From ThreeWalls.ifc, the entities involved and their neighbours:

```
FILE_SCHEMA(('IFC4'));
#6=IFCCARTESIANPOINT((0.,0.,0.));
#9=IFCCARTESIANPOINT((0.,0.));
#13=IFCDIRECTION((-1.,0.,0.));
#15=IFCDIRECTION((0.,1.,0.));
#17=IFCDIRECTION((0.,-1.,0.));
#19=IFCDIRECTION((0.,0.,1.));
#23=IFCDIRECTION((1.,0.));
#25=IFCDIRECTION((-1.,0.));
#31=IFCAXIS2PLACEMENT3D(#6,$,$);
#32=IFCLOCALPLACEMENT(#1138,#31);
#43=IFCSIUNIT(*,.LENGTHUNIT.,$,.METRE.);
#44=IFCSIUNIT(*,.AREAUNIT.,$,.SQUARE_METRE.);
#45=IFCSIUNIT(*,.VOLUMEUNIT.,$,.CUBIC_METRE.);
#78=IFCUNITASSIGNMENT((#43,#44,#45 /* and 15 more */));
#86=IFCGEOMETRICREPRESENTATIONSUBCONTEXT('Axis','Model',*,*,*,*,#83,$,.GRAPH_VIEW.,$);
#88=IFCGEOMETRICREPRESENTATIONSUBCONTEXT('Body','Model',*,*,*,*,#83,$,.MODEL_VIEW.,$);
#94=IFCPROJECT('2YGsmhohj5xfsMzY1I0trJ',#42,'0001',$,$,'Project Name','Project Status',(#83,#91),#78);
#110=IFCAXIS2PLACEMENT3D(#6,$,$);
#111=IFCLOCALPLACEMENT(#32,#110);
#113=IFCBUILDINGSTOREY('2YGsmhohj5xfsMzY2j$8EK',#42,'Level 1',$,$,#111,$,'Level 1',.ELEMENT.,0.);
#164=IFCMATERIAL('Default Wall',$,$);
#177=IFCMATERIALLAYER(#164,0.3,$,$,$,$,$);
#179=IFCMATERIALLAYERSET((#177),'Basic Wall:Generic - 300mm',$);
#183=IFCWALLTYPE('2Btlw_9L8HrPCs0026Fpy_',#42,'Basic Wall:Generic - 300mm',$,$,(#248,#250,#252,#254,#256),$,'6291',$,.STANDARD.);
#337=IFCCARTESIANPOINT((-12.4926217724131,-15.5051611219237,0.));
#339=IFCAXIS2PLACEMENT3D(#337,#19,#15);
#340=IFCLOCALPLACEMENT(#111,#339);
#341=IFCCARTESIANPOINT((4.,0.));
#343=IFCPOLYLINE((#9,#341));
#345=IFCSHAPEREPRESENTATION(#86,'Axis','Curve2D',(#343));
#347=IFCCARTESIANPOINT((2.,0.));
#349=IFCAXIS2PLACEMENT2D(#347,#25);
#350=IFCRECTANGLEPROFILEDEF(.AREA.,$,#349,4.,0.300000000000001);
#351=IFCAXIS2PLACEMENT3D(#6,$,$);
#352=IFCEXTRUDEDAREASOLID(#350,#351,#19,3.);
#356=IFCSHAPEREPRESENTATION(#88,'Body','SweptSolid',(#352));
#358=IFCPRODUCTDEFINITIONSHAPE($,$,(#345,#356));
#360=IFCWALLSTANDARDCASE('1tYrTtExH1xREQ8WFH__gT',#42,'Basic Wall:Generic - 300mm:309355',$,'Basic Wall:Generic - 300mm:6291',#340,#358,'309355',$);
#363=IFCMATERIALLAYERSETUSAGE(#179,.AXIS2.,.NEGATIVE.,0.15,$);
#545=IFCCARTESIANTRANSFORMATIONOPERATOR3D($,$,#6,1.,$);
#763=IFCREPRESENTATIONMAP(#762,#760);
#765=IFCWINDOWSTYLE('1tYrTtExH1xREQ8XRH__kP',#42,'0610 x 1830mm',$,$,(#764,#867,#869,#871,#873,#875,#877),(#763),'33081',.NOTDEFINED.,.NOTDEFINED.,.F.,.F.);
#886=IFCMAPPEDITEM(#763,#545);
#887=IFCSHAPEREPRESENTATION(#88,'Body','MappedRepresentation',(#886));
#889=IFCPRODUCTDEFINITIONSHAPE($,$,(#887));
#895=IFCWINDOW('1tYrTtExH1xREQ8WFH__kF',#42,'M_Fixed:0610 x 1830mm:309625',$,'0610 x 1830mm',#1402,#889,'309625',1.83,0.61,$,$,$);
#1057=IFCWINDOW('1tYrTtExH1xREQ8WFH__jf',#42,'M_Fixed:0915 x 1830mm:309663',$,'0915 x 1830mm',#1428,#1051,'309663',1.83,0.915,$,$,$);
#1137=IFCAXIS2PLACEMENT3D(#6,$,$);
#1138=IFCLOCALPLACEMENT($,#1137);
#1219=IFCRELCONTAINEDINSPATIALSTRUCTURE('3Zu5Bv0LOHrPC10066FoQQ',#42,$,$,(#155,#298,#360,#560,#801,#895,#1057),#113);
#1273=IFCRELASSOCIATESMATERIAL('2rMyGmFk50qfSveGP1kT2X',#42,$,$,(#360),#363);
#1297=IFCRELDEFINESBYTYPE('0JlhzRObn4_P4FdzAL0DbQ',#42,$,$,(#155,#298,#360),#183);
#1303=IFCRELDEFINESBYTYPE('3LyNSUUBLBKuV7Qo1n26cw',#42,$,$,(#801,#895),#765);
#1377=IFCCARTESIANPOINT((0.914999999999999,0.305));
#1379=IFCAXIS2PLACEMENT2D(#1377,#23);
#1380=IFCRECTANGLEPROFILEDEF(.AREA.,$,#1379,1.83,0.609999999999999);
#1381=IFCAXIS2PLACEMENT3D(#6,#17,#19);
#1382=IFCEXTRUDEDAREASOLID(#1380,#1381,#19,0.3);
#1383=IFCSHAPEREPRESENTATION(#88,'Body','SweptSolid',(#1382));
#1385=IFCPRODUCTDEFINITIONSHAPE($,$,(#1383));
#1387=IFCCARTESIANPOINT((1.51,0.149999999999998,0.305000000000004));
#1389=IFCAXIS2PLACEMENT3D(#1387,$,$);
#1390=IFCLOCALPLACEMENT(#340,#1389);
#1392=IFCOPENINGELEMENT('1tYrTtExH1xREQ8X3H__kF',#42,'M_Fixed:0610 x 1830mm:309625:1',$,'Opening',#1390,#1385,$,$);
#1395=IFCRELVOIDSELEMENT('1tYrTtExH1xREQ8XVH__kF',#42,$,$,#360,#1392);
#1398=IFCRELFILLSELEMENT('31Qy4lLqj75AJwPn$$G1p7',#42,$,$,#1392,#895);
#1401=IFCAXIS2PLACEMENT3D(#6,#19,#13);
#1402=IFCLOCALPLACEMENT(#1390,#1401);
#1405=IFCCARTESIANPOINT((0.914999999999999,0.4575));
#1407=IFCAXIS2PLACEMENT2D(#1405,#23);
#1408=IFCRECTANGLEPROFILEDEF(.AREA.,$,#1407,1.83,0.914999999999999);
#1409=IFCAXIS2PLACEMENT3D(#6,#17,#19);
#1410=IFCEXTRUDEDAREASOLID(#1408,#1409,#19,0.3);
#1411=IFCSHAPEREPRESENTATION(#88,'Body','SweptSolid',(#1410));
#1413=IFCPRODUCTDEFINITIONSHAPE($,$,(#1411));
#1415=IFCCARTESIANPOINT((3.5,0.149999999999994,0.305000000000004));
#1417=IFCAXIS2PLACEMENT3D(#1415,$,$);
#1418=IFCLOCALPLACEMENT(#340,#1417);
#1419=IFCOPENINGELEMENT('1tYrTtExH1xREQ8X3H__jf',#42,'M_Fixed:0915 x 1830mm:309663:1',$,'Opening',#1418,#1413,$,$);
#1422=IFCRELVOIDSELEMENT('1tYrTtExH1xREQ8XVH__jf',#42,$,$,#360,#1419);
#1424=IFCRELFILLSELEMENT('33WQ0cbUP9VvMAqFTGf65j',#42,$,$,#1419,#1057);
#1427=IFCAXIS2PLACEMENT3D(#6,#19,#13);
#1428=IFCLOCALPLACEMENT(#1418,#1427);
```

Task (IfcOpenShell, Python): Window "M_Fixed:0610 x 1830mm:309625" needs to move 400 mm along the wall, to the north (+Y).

```python
import ifcopenshell
import ifcopenshell.api.geometry
import ifcopenshell.util.placement

model = ifcopenshell.open("ThreeWalls.ifc")

window = model.by_guid("1tYrTtExH1xREQ8WFH__kF")
opening = window.FillsVoids[0].RelatingOpeningElement
wall = opening.VoidsElements[0].RelatingBuildingElement

wall_matrix = ifcopenshell.util.placement.get_local_placement(wall.ObjectPlacement)
shift = wall_matrix[:3, 0] * 0.4
before = ifcopenshell.util.placement.get_local_placement(window.ObjectPlacement)[:3, 3].copy()

# The window is placed relative to its opening, so it follows when the opening moves.
matrix = ifcopenshell.util.placement.get_local_placement(opening.ObjectPlacement)
matrix[:3, 3] += shift
ifcopenshell.api.geometry.edit_object_placement(
    model, product=opening, matrix=matrix, is_si=False, should_transform_children=True
)

after = ifcopenshell.util.placement.get_local_placement(window.ObjectPlacement)[:3, 3]
print("window moved by", (after - before).round(3) + 0.0)

model.write("ThreeWalls_edited.ifc")
```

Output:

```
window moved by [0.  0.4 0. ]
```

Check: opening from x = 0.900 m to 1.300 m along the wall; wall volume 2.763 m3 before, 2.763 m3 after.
